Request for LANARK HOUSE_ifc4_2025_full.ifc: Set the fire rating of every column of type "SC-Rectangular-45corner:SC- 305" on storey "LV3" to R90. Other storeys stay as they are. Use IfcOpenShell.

First a look at what the model holds.

```python
import ifcopenshell
import ifcopenshell.util.element

model = ifcopenshell.open("LANARK HOUSE_ifc4_2025_full.ifc")
print(model.schema)
storey = next(s for s in model.by_type("IfcBuildingStorey") if s.Name == "LV3")
columns = [e for e in ifcopenshell.util.element.get_decomposition(storey) if e.is_a("IfcColumn")]
seen = {}
for e in columns:
    element_type = ifcopenshell.util.element.get_type(e)
    key = (element_type.Name if element_type != e and element_type else None, ifcopenshell.util.element.get_pset(e, "Pset_ColumnCommon", "FireRating"))
    seen[key] = seen.get(key, 0) + 1
for (name, value), count in sorted(seen.items(), key=str):
    print(count, "x", name, "|", value)
```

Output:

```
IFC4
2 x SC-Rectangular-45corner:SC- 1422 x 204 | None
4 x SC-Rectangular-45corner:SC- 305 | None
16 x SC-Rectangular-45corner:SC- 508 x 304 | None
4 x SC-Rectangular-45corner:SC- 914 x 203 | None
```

```python
import ifcopenshell
import ifcopenshell.api.pset
import ifcopenshell.util.element

model = ifcopenshell.open("LANARK HOUSE_ifc4_2025_full.ifc")

storey = next(s for s in model.by_type("IfcBuildingStorey") if s.Name == "LV3")
columns = [e for e in ifcopenshell.util.element.get_decomposition(storey) if e.is_a("IfcColumn")]

count = 0
for e in columns:
    element_type = ifcopenshell.util.element.get_type(e)
    if element_type in (None, e) or element_type.Name != "SC-Rectangular-45corner:SC- 305":
        continue
    # add_pset returns the element's existing set when there is one.
    pset = ifcopenshell.api.pset.add_pset(model, product=e, name="Pset_ColumnCommon")
    ifcopenshell.api.pset.edit_pset(model, pset=pset, properties={"FireRating": "R90"})
    count += 1

print(count, "columns updated")

model.write("LANARK HOUSE_ifc4_2025_full_rev.ifc")
```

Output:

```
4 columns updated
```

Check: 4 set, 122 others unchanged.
